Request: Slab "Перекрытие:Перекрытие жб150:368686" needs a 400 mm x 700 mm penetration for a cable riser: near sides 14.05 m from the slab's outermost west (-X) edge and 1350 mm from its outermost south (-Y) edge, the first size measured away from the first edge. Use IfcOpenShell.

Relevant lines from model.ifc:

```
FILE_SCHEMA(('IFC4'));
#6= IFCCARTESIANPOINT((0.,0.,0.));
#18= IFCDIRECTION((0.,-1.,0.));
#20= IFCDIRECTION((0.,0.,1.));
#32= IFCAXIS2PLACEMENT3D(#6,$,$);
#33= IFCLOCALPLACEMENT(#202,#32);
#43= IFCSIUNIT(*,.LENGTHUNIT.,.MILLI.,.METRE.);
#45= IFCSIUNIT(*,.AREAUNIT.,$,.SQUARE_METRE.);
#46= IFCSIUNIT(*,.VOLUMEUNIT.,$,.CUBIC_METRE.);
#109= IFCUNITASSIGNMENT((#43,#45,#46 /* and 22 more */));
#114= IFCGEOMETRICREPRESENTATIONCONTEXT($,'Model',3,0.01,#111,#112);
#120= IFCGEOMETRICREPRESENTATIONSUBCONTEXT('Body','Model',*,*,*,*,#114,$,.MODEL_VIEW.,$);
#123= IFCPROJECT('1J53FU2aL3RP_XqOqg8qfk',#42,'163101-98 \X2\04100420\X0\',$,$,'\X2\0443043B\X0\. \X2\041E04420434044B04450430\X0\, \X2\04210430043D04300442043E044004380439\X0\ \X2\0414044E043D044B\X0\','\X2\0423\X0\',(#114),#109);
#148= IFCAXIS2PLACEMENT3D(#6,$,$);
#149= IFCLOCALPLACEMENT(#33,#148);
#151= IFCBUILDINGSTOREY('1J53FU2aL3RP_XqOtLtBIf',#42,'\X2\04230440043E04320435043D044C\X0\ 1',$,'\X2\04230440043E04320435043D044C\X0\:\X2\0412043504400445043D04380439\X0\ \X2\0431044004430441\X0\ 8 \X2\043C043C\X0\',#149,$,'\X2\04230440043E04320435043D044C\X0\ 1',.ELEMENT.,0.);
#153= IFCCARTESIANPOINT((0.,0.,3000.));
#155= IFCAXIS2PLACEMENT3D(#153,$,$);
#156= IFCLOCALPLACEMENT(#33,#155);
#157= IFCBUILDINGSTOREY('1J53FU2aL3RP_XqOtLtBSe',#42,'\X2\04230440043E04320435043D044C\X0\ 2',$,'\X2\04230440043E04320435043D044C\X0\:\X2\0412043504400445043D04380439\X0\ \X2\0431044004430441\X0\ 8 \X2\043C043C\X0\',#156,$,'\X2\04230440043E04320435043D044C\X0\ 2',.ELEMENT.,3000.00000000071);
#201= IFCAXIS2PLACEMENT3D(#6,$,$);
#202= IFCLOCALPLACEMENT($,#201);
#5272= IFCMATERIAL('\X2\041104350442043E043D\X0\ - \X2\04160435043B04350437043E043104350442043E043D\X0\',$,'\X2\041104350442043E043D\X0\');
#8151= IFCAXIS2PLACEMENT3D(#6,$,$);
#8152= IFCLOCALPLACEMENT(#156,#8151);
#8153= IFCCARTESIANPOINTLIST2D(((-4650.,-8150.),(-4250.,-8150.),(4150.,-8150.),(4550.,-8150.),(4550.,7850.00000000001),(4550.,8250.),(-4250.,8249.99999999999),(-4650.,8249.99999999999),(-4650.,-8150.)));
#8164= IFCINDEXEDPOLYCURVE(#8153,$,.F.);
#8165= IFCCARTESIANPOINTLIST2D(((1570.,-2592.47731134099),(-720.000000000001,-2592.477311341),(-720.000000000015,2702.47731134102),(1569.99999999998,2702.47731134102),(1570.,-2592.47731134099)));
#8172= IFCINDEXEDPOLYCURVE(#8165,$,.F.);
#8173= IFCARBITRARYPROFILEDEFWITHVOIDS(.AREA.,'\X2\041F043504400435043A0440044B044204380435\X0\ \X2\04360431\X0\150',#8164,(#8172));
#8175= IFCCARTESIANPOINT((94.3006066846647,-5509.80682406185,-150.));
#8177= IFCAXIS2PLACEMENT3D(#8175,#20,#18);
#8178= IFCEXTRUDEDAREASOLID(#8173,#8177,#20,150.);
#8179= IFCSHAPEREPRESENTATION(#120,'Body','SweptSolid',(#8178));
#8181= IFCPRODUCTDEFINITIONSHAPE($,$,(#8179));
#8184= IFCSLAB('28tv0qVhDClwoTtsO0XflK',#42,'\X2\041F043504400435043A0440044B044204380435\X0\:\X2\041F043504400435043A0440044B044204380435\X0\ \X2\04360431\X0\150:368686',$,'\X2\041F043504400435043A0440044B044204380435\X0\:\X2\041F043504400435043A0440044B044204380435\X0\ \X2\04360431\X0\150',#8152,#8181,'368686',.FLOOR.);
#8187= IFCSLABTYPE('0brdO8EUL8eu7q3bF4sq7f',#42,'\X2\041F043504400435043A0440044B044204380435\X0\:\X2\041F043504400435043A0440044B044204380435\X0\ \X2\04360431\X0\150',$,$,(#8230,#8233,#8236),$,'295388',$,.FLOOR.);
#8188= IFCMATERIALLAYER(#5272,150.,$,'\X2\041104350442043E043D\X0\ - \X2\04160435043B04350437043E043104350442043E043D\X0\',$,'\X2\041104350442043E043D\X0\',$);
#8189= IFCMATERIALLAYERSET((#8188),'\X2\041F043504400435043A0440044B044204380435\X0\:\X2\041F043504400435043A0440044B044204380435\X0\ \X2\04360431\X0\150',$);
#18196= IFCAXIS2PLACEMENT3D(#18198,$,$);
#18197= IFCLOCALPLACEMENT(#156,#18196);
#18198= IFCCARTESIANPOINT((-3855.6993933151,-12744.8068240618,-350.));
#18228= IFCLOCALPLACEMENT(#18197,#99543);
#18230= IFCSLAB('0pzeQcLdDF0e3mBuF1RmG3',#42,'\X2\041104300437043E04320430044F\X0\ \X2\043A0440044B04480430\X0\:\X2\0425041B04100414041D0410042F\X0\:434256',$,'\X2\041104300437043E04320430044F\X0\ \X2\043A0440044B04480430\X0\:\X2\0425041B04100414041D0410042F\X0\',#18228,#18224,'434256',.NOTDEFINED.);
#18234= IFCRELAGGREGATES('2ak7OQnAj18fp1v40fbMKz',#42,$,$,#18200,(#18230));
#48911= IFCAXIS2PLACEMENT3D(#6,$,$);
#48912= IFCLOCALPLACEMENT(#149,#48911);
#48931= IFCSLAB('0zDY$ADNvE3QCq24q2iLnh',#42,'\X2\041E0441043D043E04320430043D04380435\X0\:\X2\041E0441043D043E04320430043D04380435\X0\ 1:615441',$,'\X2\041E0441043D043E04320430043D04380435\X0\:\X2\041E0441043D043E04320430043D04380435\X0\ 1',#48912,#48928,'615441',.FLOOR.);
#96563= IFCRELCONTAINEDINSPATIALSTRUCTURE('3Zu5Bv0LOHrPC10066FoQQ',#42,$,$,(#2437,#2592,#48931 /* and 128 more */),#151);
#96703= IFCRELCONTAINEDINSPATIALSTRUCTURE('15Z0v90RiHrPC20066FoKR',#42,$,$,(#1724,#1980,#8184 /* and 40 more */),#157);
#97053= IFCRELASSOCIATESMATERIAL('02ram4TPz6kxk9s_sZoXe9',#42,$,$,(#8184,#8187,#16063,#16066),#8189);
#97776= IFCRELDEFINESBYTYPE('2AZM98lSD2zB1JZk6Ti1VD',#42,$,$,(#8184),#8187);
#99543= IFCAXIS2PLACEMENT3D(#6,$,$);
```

```python
import numpy as np
import ifcopenshell
import ifcopenshell.api.feature
import ifcopenshell.api.geometry
import ifcopenshell.api.root
import ifcopenshell.geom
import ifcopenshell.util.placement
import ifcopenshell.util.representation
import ifcopenshell.util.shape
import ifcopenshell.util.unit

model = ifcopenshell.open("model.ifc")
unit_scale = ifcopenshell.util.unit.calculate_unit_scale(model)
settings = ifcopenshell.geom.settings()


def volume(element):
    """Net volume in cubic metres, openings subtracted."""
    shape = ifcopenshell.geom.create_shape(settings, element)
    return ifcopenshell.util.shape.get_volume(shape.geometry)


slab = model.by_id(8184)
before = volume(slab)

# Extent in the slab's own axes, in metres. The edges named are its -X and -Y sides.
slab_shape = ifcopenshell.geom.create_shape(settings, slab)
vertices = ifcopenshell.util.shape.get_vertices(slab_shape.geometry)
x_min, y_min, bottom = vertices.min(axis=0)
top = vertices[:, 2].max()

opening = ifcopenshell.api.root.create_entity(model, ifc_class="IfcOpeningElement", name="Cable riser opening", predefined_type="OPENING")
context = ifcopenshell.util.representation.get_context(model, "Model", "Body", "MODEL_VIEW")
width, depth = 0.4, 0.7
outline = [(0.0, 0.0), (width, 0.0), (width, depth), (0.0, depth), (0.0, 0.0)]
# Overshoot both faces by 50 mm so the cut is clean.
shape = ifcopenshell.api.geometry.add_slab_representation(
    model, context=context, depth=top - bottom + 0.1, polyline=outline
)
ifcopenshell.api.geometry.assign_representation(model, product=opening, representation=shape)

matrix = ifcopenshell.util.placement.get_local_placement(slab.ObjectPlacement)
matrix[:, 3] = matrix @ np.append(np.array([x_min + 14.05, y_min + 1.35, bottom - 0.05]) / unit_scale, 1.0)
ifcopenshell.api.geometry.edit_object_placement(model, product=opening, matrix=matrix, is_si=False)
ifcopenshell.api.feature.add_feature(model, feature=opening, element=slab)

after = volume(slab)

print(f"slab volume {before:.3f} -> {after:.3f} m3")

model.write("model_updated.ifc")
```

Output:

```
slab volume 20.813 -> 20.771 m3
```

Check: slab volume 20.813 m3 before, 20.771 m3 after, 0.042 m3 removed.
